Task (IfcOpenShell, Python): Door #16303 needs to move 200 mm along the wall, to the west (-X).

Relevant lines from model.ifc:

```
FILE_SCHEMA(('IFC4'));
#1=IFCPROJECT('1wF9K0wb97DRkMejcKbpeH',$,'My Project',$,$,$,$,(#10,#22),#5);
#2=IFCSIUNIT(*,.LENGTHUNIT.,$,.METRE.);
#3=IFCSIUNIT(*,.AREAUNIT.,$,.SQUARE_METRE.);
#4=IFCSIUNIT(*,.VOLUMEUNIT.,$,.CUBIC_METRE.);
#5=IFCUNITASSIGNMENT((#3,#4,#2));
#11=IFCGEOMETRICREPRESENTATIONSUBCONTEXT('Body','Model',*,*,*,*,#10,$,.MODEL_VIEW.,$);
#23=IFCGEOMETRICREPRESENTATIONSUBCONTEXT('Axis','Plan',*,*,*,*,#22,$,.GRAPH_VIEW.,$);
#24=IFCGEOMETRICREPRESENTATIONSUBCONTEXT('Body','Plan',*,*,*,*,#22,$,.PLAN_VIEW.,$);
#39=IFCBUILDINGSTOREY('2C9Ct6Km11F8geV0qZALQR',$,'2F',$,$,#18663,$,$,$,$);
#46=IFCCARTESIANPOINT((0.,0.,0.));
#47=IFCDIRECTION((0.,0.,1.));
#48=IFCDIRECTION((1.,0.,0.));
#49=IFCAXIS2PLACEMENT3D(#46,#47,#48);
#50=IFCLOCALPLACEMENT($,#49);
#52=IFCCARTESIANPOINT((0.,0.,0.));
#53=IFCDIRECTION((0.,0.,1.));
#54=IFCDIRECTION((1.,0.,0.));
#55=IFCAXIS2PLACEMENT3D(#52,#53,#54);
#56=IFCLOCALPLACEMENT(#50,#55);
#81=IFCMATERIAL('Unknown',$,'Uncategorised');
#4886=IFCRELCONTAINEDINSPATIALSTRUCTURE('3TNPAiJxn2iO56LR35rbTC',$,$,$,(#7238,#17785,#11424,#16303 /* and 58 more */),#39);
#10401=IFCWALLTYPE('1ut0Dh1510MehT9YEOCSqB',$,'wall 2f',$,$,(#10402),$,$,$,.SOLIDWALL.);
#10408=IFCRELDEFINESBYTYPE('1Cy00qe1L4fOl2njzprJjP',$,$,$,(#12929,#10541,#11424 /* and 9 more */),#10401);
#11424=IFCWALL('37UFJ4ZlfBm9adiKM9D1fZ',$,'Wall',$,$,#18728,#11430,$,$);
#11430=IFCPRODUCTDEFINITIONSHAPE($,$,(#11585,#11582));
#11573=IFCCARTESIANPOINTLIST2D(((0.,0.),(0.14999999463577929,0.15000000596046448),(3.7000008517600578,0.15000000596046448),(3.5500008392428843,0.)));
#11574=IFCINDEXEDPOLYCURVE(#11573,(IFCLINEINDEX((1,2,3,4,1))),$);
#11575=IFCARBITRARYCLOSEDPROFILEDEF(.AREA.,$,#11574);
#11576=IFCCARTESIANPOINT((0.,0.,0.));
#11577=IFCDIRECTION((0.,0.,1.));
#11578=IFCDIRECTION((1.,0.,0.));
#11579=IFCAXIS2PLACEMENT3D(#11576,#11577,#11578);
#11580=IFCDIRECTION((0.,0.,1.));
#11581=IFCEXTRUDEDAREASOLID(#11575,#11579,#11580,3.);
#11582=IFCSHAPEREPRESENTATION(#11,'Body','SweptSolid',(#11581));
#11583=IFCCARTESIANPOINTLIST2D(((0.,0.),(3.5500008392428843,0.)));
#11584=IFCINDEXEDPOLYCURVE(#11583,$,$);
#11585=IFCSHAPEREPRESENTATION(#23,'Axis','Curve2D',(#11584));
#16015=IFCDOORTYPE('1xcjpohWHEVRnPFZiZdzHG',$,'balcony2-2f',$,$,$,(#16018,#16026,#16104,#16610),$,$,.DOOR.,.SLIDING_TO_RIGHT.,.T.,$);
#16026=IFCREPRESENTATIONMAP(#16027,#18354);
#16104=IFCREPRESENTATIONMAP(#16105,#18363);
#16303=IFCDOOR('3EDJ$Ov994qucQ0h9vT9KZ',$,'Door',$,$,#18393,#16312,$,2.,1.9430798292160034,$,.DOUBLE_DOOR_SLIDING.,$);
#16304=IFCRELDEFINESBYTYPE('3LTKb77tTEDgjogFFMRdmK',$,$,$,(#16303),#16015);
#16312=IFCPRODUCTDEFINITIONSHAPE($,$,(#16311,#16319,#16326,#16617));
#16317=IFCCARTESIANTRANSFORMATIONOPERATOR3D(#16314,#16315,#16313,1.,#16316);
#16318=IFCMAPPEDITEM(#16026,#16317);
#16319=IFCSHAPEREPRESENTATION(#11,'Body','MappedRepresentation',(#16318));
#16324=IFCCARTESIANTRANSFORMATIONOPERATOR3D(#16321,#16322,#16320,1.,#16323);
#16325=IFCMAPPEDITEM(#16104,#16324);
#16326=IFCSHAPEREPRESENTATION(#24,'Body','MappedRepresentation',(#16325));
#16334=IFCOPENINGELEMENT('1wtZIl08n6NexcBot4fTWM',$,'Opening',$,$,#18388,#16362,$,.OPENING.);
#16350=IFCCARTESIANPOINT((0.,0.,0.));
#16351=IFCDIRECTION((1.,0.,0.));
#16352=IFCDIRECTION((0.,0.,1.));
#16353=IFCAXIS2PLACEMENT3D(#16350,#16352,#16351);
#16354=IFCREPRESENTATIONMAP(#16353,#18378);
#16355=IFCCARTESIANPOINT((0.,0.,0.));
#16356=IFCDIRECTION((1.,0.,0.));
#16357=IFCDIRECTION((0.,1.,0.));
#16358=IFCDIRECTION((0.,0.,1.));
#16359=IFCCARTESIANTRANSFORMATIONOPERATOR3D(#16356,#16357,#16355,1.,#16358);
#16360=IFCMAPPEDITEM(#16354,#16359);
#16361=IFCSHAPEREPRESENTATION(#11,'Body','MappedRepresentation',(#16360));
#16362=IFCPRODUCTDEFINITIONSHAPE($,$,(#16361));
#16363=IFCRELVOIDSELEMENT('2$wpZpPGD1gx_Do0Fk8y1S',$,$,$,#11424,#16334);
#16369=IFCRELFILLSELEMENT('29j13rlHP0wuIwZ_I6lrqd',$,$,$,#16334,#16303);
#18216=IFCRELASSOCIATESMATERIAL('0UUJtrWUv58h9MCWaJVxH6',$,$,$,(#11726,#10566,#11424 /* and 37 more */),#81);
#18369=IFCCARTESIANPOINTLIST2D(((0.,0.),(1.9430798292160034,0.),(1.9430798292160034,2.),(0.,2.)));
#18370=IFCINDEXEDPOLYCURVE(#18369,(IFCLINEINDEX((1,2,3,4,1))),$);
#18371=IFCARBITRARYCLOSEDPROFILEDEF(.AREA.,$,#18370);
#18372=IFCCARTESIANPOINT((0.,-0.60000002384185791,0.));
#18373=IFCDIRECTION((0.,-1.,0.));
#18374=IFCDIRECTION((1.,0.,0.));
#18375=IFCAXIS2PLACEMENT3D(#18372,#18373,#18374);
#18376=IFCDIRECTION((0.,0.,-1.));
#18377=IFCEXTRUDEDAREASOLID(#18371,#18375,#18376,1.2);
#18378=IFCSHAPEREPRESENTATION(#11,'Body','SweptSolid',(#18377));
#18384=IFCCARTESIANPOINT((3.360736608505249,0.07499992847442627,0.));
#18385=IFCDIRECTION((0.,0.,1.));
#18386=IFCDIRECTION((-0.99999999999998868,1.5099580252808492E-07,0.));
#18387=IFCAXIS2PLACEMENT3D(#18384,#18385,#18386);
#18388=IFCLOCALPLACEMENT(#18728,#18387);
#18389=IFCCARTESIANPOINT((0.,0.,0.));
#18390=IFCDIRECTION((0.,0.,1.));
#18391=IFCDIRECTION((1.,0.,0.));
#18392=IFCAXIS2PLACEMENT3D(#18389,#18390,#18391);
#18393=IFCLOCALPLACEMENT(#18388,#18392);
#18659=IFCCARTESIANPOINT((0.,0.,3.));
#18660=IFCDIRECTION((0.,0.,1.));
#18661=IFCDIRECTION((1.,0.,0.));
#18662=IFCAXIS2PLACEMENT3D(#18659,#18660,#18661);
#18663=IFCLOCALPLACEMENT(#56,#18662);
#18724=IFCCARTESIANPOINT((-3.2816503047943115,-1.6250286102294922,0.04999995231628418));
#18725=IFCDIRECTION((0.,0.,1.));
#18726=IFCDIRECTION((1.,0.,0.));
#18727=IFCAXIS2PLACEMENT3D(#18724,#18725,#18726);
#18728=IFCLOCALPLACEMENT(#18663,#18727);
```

```python
import ifcopenshell
import ifcopenshell.api.geometry
import ifcopenshell.util.placement

model = ifcopenshell.open("model.ifc")

door = model.by_id(16303)
opening = door.FillsVoids[0].RelatingOpeningElement
wall = opening.VoidsElements[0].RelatingBuildingElement

wall_matrix = ifcopenshell.util.placement.get_local_placement(wall.ObjectPlacement)
shift = wall_matrix[:3, 0] * -0.2
before = ifcopenshell.util.placement.get_local_placement(door.ObjectPlacement)[:3, 3].copy()

# The door is placed relative to its opening, so it follows when the opening moves.
matrix = ifcopenshell.util.placement.get_local_placement(opening.ObjectPlacement)
matrix[:3, 3] += shift
ifcopenshell.api.geometry.edit_object_placement(
    model, product=opening, matrix=matrix, is_si=False, should_transform_children=True
)

after = ifcopenshell.util.placement.get_local_placement(door.ObjectPlacement)[:3, 3]
print("door moved by", (after - before).round(3) + 0.0)

model.write("model_edited.ifc")
```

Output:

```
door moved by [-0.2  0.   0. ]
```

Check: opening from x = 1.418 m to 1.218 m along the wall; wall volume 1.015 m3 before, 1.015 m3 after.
